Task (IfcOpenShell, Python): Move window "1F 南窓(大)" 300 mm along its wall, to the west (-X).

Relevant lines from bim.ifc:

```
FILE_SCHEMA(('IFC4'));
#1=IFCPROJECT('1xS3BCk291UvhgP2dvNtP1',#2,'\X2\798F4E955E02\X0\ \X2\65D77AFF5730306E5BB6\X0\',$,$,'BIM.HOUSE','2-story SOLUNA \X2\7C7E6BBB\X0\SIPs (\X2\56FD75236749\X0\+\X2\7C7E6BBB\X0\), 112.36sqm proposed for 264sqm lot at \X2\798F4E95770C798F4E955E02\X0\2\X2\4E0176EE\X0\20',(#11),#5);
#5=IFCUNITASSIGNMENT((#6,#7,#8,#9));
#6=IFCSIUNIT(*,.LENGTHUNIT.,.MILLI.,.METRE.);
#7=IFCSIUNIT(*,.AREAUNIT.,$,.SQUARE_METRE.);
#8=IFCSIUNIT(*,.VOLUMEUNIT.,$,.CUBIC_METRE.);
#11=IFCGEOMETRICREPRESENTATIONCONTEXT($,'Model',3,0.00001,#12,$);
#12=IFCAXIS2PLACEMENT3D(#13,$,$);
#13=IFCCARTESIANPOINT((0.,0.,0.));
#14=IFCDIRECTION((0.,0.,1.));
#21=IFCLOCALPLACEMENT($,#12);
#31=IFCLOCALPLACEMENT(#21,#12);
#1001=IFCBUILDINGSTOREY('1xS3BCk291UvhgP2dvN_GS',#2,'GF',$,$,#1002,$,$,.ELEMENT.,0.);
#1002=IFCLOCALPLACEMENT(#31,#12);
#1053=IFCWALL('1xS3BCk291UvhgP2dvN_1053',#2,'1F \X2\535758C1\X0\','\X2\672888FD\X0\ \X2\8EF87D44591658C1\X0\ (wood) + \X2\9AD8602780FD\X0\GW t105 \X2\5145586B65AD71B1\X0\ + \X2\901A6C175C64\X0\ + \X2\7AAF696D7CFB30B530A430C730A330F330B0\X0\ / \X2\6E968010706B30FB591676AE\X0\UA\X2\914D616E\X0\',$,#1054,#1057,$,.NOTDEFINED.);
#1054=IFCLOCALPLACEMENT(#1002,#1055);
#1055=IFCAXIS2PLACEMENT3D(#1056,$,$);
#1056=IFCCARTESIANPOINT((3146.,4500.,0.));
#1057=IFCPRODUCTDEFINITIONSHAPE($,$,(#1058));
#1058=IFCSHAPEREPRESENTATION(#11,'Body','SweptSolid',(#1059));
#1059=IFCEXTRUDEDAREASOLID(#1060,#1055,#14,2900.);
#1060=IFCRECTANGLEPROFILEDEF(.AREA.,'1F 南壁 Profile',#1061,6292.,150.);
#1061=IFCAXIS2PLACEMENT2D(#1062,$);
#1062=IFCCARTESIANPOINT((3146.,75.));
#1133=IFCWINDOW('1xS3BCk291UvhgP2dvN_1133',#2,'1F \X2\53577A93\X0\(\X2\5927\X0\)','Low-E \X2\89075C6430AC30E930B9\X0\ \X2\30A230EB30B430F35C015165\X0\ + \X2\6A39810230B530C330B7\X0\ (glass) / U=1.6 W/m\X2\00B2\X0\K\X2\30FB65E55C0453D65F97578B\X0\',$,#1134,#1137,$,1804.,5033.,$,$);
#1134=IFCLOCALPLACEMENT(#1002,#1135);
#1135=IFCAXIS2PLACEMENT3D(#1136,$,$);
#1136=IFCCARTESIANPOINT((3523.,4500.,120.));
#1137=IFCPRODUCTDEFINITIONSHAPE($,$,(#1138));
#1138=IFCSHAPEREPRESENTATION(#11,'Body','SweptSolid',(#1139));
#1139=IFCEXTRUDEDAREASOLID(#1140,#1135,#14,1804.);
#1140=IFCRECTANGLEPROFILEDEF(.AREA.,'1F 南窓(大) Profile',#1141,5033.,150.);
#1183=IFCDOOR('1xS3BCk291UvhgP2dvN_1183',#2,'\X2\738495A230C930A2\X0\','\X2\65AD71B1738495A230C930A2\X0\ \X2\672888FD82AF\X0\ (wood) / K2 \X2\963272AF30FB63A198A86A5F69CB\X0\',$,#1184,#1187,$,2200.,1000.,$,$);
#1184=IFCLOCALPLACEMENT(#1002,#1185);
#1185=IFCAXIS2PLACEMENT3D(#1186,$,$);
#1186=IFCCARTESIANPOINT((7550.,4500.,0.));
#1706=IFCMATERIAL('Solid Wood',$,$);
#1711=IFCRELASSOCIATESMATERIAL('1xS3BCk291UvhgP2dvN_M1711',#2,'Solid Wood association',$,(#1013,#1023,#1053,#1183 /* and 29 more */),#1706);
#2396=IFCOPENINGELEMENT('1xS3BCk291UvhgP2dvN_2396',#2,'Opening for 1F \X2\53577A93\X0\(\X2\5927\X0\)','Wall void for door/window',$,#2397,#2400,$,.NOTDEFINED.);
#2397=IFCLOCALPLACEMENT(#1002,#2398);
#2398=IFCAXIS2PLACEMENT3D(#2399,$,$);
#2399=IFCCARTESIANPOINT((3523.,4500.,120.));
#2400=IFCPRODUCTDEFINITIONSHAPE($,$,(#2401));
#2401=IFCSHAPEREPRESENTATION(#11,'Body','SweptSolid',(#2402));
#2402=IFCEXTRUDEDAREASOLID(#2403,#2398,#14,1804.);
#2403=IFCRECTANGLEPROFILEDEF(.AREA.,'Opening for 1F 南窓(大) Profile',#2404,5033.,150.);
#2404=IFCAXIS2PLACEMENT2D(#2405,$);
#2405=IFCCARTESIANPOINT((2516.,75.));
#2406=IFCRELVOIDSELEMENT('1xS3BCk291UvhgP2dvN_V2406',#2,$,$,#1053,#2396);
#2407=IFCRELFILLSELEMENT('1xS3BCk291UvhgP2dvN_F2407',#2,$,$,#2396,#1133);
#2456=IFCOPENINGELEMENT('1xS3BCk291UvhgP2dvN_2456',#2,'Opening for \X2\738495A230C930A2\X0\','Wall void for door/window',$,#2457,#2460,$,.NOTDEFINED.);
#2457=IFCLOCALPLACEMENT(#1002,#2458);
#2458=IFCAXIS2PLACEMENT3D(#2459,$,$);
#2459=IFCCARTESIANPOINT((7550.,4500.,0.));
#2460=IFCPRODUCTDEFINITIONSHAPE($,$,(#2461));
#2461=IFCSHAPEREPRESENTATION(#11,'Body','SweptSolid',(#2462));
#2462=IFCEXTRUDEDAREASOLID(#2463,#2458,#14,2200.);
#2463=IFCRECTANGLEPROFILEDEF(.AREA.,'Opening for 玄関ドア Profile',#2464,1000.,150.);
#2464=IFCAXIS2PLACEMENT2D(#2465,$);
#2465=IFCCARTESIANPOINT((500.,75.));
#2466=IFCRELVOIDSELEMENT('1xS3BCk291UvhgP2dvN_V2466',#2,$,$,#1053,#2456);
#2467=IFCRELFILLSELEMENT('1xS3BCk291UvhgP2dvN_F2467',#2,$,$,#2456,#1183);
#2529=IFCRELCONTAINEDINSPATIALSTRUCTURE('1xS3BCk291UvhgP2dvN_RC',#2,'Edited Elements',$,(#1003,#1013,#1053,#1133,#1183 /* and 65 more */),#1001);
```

```python
import ifcopenshell
import ifcopenshell.api.geometry
import ifcopenshell.util.placement
import ifcopenshell.util.unit

model = ifcopenshell.open("bim.ifc")
unit_scale = ifcopenshell.util.unit.calculate_unit_scale(model)

window = model.by_guid("1xS3BCk291UvhgP2dvN_1133")
opening = window.FillsVoids[0].RelatingOpeningElement
wall = opening.VoidsElements[0].RelatingBuildingElement

wall_matrix = ifcopenshell.util.placement.get_local_placement(wall.ObjectPlacement)
shift = wall_matrix[:3, 0] * -0.3 / unit_scale
before = ifcopenshell.util.placement.get_local_placement(window.ObjectPlacement)[:3, 3].copy()

# The window is not placed relative to its opening, so move both.
for product in (opening, window):
    matrix = ifcopenshell.util.placement.get_local_placement(product.ObjectPlacement)
    matrix[:3, 3] += shift
    ifcopenshell.api.geometry.edit_object_placement(model, product=product, matrix=matrix, is_si=False)

after = ifcopenshell.util.placement.get_local_placement(window.ObjectPlacement)[:3, 3]
print("window moved by", (after - before).round(3) + 0.0)

model.write("bim-out.ifc")
```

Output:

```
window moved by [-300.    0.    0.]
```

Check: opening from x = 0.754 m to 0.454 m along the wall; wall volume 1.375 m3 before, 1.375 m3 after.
